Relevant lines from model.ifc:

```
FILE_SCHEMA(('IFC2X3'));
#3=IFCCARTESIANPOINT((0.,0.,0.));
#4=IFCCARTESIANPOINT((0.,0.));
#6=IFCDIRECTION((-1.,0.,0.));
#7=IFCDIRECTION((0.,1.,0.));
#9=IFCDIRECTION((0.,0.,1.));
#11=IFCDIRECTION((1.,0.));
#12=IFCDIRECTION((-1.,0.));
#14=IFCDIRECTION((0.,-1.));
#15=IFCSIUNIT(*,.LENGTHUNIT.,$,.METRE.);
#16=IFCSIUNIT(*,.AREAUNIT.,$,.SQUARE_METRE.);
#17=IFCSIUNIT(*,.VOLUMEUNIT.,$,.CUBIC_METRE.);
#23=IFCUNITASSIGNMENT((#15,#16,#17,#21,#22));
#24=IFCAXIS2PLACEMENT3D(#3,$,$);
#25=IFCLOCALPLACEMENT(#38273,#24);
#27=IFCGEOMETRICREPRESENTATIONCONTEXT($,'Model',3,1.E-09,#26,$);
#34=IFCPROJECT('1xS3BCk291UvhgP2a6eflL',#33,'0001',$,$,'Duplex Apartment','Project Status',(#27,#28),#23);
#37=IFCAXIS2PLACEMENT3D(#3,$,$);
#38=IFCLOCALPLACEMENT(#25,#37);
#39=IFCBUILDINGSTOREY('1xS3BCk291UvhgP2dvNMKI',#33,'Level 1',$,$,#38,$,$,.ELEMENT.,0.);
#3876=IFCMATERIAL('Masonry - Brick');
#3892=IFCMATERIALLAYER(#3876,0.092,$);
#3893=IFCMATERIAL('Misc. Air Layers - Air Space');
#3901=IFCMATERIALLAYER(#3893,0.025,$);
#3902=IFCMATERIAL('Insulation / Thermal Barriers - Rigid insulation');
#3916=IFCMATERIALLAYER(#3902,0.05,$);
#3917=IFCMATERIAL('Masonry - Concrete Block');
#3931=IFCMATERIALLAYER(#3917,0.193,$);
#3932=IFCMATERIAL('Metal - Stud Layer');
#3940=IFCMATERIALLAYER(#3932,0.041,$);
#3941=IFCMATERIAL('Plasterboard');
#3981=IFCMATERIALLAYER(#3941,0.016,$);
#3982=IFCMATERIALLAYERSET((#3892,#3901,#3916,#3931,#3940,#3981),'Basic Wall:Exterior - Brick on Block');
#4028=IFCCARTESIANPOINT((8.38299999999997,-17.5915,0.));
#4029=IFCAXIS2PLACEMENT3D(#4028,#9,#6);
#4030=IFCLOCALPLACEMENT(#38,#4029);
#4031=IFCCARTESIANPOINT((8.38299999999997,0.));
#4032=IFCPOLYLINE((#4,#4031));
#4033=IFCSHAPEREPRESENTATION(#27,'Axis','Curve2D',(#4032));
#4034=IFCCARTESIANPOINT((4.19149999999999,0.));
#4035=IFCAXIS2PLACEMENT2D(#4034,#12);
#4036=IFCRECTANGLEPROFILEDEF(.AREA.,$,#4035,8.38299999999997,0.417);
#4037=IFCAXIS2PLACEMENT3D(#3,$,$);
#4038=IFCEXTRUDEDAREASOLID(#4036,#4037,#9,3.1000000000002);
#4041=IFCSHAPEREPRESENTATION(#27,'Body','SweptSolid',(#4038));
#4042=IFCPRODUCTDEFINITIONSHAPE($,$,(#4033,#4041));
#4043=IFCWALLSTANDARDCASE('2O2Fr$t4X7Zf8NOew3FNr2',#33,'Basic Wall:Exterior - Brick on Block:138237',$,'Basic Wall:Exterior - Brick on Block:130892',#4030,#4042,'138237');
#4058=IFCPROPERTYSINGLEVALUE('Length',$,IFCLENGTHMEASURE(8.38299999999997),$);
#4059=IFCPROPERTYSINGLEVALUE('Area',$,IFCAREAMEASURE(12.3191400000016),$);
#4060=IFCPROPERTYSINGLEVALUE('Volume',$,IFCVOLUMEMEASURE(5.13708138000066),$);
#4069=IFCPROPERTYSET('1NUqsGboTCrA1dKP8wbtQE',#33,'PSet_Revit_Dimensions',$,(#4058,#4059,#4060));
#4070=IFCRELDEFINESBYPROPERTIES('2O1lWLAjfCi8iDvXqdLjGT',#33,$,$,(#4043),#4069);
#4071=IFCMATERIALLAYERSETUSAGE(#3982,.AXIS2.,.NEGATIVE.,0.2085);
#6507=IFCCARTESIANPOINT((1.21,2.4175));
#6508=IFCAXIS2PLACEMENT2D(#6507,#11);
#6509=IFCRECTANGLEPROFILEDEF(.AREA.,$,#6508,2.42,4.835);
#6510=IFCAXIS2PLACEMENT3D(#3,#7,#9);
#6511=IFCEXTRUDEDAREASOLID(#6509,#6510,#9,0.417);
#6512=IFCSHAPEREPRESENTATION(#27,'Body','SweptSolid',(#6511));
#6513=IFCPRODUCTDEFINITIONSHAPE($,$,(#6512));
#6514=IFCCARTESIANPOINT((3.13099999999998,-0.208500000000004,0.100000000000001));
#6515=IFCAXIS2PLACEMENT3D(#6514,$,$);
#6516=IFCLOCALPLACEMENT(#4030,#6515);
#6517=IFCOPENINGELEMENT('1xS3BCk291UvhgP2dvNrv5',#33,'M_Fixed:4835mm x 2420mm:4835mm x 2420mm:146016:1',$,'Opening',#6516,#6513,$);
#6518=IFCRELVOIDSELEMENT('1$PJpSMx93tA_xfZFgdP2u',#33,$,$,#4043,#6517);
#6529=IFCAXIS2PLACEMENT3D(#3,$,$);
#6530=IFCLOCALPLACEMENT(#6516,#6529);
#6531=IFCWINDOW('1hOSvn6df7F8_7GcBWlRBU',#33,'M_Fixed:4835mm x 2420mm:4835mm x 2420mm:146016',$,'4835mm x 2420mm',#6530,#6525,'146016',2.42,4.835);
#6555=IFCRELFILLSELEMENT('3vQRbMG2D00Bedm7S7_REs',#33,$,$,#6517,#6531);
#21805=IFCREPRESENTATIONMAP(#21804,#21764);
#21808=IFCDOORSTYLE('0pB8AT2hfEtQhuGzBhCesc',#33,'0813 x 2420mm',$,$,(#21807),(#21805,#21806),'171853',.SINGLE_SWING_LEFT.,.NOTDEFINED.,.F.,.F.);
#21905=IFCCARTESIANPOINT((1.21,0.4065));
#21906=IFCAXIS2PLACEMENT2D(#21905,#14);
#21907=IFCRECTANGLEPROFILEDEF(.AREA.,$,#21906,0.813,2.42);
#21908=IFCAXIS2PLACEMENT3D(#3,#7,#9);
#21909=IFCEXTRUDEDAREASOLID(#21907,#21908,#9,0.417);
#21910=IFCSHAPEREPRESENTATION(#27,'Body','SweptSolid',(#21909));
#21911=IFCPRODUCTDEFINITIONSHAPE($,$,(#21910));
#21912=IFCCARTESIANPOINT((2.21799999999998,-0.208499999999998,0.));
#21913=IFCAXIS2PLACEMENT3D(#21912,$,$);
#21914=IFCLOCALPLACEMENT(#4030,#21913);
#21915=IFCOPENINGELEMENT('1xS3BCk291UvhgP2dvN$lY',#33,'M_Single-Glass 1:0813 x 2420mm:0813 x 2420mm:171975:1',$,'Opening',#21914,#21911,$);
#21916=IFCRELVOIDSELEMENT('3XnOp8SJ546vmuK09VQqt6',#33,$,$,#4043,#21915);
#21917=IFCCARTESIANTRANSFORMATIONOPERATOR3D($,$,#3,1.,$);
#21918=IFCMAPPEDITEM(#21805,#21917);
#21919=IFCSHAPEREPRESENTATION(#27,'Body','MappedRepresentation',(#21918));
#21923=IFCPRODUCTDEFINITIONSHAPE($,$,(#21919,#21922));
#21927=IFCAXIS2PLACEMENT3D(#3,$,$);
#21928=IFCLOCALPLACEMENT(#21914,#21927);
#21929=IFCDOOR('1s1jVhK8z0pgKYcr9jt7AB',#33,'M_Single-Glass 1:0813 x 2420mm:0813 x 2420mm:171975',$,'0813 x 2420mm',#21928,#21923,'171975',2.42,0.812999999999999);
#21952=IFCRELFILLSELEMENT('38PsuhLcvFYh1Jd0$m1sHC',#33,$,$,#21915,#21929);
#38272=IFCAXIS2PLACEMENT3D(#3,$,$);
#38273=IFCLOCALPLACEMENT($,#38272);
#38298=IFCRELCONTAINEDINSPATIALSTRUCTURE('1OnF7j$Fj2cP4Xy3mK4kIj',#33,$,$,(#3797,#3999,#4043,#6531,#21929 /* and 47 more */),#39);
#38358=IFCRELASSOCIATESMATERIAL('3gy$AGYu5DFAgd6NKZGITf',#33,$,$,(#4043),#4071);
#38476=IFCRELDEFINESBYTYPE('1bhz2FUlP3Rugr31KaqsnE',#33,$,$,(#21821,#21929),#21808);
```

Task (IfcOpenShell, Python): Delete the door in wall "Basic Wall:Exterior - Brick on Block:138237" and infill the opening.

```python
import ifcopenshell
import ifcopenshell.api.feature
import ifcopenshell.api.pset
import ifcopenshell.api.root
import ifcopenshell.geom
import ifcopenshell.util.element
import ifcopenshell.util.shape
import ifcopenshell.util.unit

model = ifcopenshell.open("model.ifc")
area_scale = ifcopenshell.util.unit.calculate_unit_scale(model, "AREAUNIT")
volume_scale = ifcopenshell.util.unit.calculate_unit_scale(model, "VOLUMEUNIT")
settings = ifcopenshell.geom.settings()


def volume(element):
    """Net volume in cubic metres, openings subtracted."""
    shape = ifcopenshell.geom.create_shape(settings, element)
    return ifcopenshell.util.shape.get_volume(shape.geometry)


door = model.by_id(21929)
opening = door.FillsVoids[0].RelatingOpeningElement
wall = opening.VoidsElements[0].RelatingBuildingElement
before = volume(wall)

ifcopenshell.api.root.remove_product(model, product=door)
ifcopenshell.api.feature.remove_feature(model, feature=opening)

after = volume(wall)
thickness = 0.417  # wall thickness in metres

# Update the wall's stored quantities.
pset = model.by_id(ifcopenshell.util.element.get_pset(wall, "PSet_Revit_Dimensions", should_inherit=False)["id"])
ifcopenshell.api.pset.edit_pset(model, pset=pset, properties={
    "Area": model.create_entity("IfcAreaMeasure", after / thickness / area_scale),
    "Volume": model.create_entity("IfcVolumeMeasure", after / volume_scale),
})

print(f"wall volume {before:.3f} -> {after:.3f} m3")

model.write("model_rev.ifc")
```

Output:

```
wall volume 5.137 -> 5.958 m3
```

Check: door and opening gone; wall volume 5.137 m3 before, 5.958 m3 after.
